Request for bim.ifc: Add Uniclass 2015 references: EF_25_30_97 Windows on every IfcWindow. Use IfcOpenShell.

First a look at what the model holds.

```python
import ifcopenshell

model = ifcopenshell.open("bim.ifc")
print(model.schema)
print("classifications:", [c.Name for c in model.by_type("IfcClassification")])
for ifc_class in ("IfcDoor", "IfcRoof", "IfcStair", "IfcWall", "IfcWindow"):
    print(ifc_class, len(model.by_type(ifc_class)))
```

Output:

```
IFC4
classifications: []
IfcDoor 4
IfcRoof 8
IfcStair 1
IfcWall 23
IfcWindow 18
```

```python
import ifcopenshell
import ifcopenshell.api.classification

model = ifcopenshell.open("bim.ifc")

system = ifcopenshell.api.classification.add_classification(model, classification="Uniclass 2015")

codes = {
    "IfcWindow": ("EF_25_30_97", "Windows"),
}
for ifc_class, (code, name) in codes.items():
    products = model.by_type(ifc_class)
    ifcopenshell.api.classification.add_reference(
        model, products=products, classification=system, identification=code, name=name
    )
    print(code, len(products))

model.write("bim-out.ifc")
```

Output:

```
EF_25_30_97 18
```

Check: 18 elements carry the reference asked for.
